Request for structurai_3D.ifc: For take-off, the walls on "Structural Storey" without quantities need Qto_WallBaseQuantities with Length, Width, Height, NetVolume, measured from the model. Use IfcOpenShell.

First a look at what the model holds.

```python
import ifcopenshell
import ifcopenshell.util.element
import ifcopenshell.util.unit

model = ifcopenshell.open("structurai_3D.ifc")
print(model.schema)
for unit_type in ("LENGTHUNIT", "AREAUNIT", "VOLUMEUNIT"):
    print(unit_type, ifcopenshell.util.unit.calculate_unit_scale(model, unit_type))
storey = next(s for s in model.by_type("IfcBuildingStorey") if s.Name == "Structural Storey")
walls = [e for e in ifcopenshell.util.element.get_decomposition(storey) if e.is_a("IfcWall")]
for e in sorted(walls, key=lambda e: e.id()):
    print(e.id(), e.is_a(), e.Name, list(ifcopenshell.util.element.get_psets(e, qtos_only=True)), sep=" | ")
```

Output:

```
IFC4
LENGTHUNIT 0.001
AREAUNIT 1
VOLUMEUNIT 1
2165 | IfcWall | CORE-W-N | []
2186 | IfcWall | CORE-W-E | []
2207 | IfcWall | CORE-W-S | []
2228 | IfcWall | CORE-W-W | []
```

```python
import ifcopenshell
import ifcopenshell.api.pset
import ifcopenshell.geom
import ifcopenshell.util.element
import ifcopenshell.util.shape
import ifcopenshell.util.unit

model = ifcopenshell.open("structurai_3D.ifc")
unit_scale = ifcopenshell.util.unit.calculate_unit_scale(model)
volume_scale = ifcopenshell.util.unit.calculate_unit_scale(model, "VOLUMEUNIT")
settings = ifcopenshell.geom.settings()

storey = next(s for s in model.by_type("IfcBuildingStorey") if s.Name == "Structural Storey")
walls = [e for e in ifcopenshell.util.element.get_decomposition(storey) if e.is_a("IfcWall")]

for e in sorted(walls, key=lambda e: e.id()):
    if ifcopenshell.util.element.get_psets(e, qtos_only=True, should_inherit=False):
        continue
    # Geometry comes back in metres, in the element's own axes.
    shape = ifcopenshell.geom.create_shape(settings, e)
    values = {
        "Length": ifcopenshell.util.shape.get_x(shape.geometry) / unit_scale,
        "Width": ifcopenshell.util.shape.get_y(shape.geometry) / unit_scale,
        "Height": ifcopenshell.util.shape.get_z(shape.geometry) / unit_scale,
        "NetVolume": ifcopenshell.util.shape.get_volume(shape.geometry) / volume_scale,
    }
    qto = ifcopenshell.api.pset.add_qto(model, product=e, name="Qto_WallBaseQuantities")
    ifcopenshell.api.pset.edit_qto(model, qto=qto, properties=values)
    print(e.id(), {k: round(v, 3) for k, v in values.items()})

model.write("structurai_3D_v2.ifc")
```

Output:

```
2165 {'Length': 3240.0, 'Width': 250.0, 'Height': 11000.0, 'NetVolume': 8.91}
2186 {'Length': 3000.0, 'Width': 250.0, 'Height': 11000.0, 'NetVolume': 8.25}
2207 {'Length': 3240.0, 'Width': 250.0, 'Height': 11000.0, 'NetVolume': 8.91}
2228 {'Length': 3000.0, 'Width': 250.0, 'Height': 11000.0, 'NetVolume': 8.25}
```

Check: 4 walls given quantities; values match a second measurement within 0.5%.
